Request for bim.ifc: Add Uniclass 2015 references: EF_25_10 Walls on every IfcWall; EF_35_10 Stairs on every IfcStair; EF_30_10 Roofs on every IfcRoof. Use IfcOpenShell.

First a look at what the model holds.

```python
import ifcopenshell

model = ifcopenshell.open("bim.ifc")
print(model.schema)
print("classifications:", [c.Name for c in model.by_type("IfcClassification")])
for ifc_class in ("IfcDoor", "IfcRoof", "IfcStair", "IfcWall", "IfcWindow"):
    print(ifc_class, len(model.by_type(ifc_class)))
```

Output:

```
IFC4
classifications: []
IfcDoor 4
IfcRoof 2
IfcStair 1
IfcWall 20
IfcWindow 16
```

```python
import ifcopenshell
import ifcopenshell.api.classification

model = ifcopenshell.open("bim.ifc")

system = ifcopenshell.api.classification.add_classification(model, classification="Uniclass 2015")

codes = {
    "IfcWall": ("EF_25_10", "Walls"),
    "IfcStair": ("EF_35_10", "Stairs"),
    "IfcRoof": ("EF_30_10", "Roofs"),
}
for ifc_class, (code, name) in codes.items():
    products = model.by_type(ifc_class)
    ifcopenshell.api.classification.add_reference(
        model, products=products, classification=system, identification=code, name=name
    )
    print(code, len(products))

model.write("bim_updated.ifc")
```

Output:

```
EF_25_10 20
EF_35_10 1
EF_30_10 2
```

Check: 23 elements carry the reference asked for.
